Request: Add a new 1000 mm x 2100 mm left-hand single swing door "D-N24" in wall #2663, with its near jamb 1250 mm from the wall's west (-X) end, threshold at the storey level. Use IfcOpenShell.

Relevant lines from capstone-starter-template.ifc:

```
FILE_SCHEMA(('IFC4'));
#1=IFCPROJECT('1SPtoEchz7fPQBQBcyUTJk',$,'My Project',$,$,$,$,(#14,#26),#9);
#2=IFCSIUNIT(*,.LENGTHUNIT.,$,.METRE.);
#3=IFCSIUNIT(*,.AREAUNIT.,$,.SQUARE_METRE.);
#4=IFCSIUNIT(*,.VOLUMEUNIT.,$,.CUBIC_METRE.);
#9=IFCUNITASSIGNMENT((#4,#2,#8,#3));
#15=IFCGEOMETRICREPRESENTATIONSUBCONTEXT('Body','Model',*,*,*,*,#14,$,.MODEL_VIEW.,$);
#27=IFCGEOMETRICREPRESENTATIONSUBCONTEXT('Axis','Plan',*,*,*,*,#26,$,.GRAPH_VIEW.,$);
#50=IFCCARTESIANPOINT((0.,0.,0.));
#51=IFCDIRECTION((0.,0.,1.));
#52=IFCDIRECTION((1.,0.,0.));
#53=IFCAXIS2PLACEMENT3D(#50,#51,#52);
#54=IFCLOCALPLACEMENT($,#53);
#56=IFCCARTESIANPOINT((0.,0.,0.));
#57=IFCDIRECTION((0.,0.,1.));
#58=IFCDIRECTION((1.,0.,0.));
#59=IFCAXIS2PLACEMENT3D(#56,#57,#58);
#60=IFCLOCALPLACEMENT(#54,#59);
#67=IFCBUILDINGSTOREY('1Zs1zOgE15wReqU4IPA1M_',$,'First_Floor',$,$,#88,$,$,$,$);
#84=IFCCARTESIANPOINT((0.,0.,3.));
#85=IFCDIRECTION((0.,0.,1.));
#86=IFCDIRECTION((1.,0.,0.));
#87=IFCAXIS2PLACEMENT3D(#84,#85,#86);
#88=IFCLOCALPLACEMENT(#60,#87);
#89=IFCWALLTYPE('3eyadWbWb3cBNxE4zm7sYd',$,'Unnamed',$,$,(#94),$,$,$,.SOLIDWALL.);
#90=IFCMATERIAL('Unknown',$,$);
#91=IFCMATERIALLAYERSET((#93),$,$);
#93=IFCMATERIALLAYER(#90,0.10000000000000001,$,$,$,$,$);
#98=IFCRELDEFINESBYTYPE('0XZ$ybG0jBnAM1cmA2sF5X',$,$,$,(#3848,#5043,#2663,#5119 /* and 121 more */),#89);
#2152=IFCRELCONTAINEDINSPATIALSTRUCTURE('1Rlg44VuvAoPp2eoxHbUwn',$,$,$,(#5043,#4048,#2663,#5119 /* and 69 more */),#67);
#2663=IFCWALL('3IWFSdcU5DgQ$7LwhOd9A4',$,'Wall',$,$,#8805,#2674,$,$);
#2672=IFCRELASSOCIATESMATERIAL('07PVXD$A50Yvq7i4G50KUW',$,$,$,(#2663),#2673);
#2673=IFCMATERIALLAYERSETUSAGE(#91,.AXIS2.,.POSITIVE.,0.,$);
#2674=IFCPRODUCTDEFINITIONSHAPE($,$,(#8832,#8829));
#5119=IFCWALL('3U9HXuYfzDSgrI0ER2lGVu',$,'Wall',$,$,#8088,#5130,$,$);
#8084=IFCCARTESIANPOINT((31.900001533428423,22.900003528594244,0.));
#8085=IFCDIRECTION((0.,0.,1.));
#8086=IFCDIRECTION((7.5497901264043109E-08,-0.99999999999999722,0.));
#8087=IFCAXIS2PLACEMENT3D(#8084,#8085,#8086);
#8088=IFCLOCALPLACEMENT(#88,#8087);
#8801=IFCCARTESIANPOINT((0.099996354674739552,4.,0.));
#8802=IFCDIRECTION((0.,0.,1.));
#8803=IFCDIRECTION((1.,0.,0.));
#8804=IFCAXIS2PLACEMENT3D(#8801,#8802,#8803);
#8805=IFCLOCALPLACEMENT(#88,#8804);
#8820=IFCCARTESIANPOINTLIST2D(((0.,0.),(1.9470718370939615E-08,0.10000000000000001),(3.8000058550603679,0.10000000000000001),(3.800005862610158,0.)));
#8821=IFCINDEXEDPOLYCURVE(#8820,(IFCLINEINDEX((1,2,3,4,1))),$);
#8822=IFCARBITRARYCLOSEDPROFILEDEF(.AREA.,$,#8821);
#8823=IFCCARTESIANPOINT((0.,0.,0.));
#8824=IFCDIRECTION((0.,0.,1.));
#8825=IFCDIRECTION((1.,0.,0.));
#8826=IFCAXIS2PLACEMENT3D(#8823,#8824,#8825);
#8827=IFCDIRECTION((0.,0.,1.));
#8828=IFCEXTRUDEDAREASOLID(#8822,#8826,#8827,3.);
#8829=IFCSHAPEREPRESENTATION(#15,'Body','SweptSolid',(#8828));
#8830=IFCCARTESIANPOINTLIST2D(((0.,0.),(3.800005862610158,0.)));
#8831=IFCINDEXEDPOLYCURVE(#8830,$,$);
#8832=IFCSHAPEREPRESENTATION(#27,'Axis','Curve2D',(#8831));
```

```python
import numpy as np
import ifcopenshell
import ifcopenshell.api.feature
import ifcopenshell.api.geometry
import ifcopenshell.api.root
import ifcopenshell.api.spatial
import ifcopenshell.geom
import ifcopenshell.util.element
import ifcopenshell.util.placement
import ifcopenshell.util.representation
import ifcopenshell.util.shape
import ifcopenshell.util.unit

model = ifcopenshell.open("capstone-starter-template.ifc")
unit_scale = ifcopenshell.util.unit.calculate_unit_scale(model)
settings = ifcopenshell.geom.settings()


def volume(element):
    """Net volume in cubic metres, openings subtracted."""
    shape = ifcopenshell.geom.create_shape(settings, element)
    return ifcopenshell.util.shape.get_volume(shape.geometry)


wall = model.by_guid("3IWFSdcU5DgQ$7LwhOd9A4")
storey = ifcopenshell.util.element.get_container(wall, ifc_class="IfcBuildingStorey")
context = ifcopenshell.util.representation.get_context(model, "Model", "Body", "MODEL_VIEW")
before = volume(wall)

width, height, from_end, sill = 1, 2.1, 1.25, 0.0  # metres

# The wall runs along its own X axis, and the end named is its -X end.
wall_shape = ifcopenshell.geom.create_shape(settings, wall)
x, y, z = ifcopenshell.util.shape.get_vertices(wall_shape.geometry).T
start = x.min() + from_end
face, thickness = float(y.min()), float(y.max() - y.min())
wall_matrix = ifcopenshell.util.placement.get_local_placement(wall.ObjectPlacement)
level = ifcopenshell.util.placement.get_local_placement(storey.ObjectPlacement)[2, 3]


def in_wall(x, y):
    """Placement at x, y metres in the wall's axes, at sill height."""
    matrix = wall_matrix.copy()
    matrix[:, 3] = wall_matrix @ np.array([x / unit_scale, y / unit_scale, 0.0, 1.0])
    matrix[2, 3] = level + sill / unit_scale
    return matrix


# Opening: a box that overshoots both wall faces by 50 mm.
opening = ifcopenshell.api.root.create_entity(model, ifc_class="IfcOpeningElement", predefined_type="OPENING")
box = ifcopenshell.api.geometry.add_wall_representation(
    model, context=context, length=width, height=height, thickness=thickness + 0.1
)
ifcopenshell.api.geometry.assign_representation(model, product=opening, representation=box)
ifcopenshell.api.geometry.edit_object_placement(model, product=opening, matrix=in_wall(start, face - 0.05), is_si=False)
ifcopenshell.api.feature.add_feature(model, feature=opening, element=wall)

door = ifcopenshell.api.root.create_entity(model, ifc_class="IfcDoor", name="D-N24", predefined_type="DOOR")
door.OverallWidth, door.OverallHeight = width / unit_scale, height / unit_scale
door.OperationType = "SINGLE_SWING_LEFT"
body = ifcopenshell.api.geometry.add_door_representation(
    model,
    context=context,
    overall_width=door.OverallWidth,
    overall_height=door.OverallHeight,
    operation_type="SINGLE_SWING_LEFT",
    lining_properties={"LiningDepth": thickness / unit_scale, "ThresholdDepth": thickness / unit_scale},
)
ifcopenshell.api.geometry.assign_representation(model, product=door, representation=body)
ifcopenshell.api.spatial.assign_container(model, products=[door], relating_structure=storey)
ifcopenshell.api.feature.add_filling(model, opening=opening, element=door)

# The lining spans the wall, so the door starts at the wall face.
ifcopenshell.api.geometry.edit_object_placement(model, product=door, matrix=in_wall(start, face), is_si=False)

after = volume(wall)

print(f"wall volume {before:.3f} -> {after:.3f} m3")

model.write("capstone-starter-template_v2.ifc")
```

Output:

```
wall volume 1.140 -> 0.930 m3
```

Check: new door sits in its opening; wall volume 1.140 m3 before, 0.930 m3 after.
